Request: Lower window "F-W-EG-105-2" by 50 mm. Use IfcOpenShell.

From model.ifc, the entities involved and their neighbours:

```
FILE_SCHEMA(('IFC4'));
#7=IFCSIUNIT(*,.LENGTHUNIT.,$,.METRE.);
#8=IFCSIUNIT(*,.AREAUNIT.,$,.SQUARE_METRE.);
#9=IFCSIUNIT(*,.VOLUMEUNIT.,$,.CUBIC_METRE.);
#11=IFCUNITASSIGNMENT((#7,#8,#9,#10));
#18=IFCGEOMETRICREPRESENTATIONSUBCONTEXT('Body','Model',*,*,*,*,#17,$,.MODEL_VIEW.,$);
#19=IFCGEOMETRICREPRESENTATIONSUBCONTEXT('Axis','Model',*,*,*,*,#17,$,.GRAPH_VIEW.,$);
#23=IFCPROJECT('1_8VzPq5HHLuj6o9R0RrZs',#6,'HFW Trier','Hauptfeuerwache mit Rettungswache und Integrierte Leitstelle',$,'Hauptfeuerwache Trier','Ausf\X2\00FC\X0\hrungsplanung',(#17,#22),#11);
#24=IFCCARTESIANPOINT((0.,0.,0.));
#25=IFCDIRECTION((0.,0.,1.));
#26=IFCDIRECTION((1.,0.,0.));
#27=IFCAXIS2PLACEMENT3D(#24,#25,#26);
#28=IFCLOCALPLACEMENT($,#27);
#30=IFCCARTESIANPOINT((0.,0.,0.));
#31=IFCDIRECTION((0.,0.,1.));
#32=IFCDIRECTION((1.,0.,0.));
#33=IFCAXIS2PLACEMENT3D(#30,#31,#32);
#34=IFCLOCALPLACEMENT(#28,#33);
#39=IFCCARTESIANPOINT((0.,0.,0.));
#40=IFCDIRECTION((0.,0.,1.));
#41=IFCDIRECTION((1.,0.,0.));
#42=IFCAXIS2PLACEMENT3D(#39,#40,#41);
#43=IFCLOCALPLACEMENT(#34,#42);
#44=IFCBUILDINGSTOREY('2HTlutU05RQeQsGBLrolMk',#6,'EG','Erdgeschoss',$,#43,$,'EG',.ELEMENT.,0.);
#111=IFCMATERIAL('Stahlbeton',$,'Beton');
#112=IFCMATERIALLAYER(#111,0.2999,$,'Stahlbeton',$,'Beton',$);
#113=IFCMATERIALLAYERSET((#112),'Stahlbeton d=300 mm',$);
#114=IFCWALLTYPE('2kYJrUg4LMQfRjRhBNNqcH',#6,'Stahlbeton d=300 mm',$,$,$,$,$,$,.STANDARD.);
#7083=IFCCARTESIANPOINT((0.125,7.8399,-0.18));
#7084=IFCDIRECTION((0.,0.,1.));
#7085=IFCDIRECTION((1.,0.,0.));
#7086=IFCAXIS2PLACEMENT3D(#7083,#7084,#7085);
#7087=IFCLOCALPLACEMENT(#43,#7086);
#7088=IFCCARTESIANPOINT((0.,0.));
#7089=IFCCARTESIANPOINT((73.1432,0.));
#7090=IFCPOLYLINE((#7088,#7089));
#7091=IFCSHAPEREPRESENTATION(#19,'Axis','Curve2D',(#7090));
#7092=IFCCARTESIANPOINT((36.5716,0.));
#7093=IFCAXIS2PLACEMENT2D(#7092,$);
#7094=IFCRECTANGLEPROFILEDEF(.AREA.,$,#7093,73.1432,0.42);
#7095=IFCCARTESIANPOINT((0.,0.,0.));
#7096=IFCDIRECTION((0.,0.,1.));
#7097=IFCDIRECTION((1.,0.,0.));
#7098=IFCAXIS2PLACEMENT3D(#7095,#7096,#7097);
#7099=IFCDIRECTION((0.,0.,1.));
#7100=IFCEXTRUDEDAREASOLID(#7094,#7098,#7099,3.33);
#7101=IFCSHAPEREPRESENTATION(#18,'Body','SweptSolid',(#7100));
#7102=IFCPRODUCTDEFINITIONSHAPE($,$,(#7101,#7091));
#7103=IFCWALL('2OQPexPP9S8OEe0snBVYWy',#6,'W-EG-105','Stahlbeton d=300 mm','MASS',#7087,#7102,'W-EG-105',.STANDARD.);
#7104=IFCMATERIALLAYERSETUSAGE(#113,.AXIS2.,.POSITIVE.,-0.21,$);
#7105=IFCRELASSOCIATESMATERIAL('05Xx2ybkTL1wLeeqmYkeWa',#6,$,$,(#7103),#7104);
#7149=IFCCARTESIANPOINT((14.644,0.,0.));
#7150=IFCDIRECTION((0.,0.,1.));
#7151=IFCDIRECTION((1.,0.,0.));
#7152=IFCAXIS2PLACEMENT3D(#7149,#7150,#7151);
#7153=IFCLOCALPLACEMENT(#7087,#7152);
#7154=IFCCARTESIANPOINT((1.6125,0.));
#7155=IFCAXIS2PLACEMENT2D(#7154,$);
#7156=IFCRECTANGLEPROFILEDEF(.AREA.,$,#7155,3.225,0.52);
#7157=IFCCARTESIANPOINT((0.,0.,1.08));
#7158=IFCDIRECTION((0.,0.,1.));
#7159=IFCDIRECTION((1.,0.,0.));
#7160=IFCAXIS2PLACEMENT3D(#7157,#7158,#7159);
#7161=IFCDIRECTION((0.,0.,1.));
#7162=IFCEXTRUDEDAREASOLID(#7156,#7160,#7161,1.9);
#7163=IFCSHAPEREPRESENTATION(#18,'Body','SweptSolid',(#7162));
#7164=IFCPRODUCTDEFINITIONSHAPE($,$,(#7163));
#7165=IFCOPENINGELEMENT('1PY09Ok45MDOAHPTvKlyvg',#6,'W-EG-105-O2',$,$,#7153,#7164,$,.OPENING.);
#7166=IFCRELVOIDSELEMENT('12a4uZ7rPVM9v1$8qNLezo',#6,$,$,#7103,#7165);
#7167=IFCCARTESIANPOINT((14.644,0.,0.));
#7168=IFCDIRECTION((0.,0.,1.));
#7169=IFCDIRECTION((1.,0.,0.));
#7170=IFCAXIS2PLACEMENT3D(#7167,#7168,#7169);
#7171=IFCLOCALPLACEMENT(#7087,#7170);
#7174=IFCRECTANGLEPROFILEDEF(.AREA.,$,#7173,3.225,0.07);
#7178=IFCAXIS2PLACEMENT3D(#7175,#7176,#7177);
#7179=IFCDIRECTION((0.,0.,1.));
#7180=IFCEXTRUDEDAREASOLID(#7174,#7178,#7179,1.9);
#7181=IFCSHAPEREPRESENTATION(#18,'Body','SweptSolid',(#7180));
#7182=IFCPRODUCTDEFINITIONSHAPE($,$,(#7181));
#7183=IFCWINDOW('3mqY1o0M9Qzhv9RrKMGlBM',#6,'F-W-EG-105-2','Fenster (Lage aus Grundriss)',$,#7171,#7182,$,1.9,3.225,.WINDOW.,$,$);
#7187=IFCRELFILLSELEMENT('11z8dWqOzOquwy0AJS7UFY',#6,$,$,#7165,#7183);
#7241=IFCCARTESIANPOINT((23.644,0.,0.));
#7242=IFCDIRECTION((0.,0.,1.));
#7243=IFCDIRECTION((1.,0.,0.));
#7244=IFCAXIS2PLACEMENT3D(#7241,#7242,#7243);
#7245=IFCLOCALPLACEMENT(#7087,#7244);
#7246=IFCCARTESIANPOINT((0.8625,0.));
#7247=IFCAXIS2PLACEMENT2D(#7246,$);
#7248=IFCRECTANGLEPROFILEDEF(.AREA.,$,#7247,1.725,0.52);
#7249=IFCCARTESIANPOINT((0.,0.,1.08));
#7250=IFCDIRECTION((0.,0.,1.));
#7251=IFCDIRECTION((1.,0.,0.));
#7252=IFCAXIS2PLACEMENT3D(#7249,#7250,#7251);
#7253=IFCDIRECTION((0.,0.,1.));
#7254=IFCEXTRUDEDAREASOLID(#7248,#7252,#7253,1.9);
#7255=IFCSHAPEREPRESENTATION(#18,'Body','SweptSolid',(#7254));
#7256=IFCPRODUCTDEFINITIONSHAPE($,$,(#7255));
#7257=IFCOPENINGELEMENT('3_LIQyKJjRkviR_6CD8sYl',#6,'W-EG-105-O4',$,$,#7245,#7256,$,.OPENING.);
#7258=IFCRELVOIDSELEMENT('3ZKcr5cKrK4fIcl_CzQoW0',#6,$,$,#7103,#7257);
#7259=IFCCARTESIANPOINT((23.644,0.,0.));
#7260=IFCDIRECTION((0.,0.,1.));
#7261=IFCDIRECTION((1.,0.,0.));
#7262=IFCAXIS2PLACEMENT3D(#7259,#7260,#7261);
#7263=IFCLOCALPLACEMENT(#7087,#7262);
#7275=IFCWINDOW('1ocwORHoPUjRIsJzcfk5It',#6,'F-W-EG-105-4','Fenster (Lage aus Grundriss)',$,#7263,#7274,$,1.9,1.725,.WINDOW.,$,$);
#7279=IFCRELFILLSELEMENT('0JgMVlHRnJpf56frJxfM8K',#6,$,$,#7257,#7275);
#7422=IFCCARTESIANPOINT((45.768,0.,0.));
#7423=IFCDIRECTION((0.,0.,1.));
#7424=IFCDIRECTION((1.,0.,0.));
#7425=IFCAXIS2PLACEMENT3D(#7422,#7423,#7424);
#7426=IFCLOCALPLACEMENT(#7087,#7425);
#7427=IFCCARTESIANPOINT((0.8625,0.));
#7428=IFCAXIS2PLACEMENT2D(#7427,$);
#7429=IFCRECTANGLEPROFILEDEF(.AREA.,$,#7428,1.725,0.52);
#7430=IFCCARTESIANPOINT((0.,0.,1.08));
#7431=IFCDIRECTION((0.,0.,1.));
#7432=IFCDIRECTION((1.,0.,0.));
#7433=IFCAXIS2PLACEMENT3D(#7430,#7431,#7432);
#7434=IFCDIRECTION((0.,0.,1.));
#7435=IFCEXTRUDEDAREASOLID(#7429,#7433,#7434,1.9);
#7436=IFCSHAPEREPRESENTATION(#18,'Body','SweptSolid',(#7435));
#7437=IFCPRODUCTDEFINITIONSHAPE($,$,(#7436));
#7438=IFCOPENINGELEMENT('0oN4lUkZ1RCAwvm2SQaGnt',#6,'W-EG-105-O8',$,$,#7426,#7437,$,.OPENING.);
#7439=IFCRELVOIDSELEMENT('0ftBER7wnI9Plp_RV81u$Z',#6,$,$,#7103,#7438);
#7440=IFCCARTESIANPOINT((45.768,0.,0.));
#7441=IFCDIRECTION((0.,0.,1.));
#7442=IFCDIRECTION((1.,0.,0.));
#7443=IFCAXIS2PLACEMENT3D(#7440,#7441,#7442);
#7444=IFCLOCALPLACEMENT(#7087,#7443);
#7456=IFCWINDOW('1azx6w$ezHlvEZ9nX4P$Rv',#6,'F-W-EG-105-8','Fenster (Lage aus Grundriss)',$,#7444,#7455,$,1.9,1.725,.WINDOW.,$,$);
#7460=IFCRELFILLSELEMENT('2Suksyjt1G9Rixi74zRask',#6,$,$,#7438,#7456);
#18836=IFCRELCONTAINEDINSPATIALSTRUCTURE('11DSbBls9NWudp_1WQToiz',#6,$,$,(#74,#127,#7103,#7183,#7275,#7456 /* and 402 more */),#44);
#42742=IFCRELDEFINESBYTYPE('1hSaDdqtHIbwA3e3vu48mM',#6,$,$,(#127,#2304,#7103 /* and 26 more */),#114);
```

```python
import numpy as np
import ifcopenshell
import ifcopenshell.api.geometry
import ifcopenshell.util.placement
import ifcopenshell.util.unit

model = ifcopenshell.open("model.ifc")
unit_scale = ifcopenshell.util.unit.calculate_unit_scale(model)

window = model.by_guid("3mqY1o0M9Qzhv9RrKMGlBM")
opening = window.FillsVoids[0].RelatingOpeningElement
dz = -0.05

shift = np.array([0.0, 0.0, dz])
# The window is not placed relative to its opening, so move both.
for product in (opening, window):
    matrix = ifcopenshell.util.placement.get_local_placement(product.ObjectPlacement)
    matrix[:3, 3] += shift
    ifcopenshell.api.geometry.edit_object_placement(model, product=product, matrix=matrix, is_si=False)

print(f"moved by {dz * unit_scale:+.3f} m")

model.write("model_edited.ifc")
```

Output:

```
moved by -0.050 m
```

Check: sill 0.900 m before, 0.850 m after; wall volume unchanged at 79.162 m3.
